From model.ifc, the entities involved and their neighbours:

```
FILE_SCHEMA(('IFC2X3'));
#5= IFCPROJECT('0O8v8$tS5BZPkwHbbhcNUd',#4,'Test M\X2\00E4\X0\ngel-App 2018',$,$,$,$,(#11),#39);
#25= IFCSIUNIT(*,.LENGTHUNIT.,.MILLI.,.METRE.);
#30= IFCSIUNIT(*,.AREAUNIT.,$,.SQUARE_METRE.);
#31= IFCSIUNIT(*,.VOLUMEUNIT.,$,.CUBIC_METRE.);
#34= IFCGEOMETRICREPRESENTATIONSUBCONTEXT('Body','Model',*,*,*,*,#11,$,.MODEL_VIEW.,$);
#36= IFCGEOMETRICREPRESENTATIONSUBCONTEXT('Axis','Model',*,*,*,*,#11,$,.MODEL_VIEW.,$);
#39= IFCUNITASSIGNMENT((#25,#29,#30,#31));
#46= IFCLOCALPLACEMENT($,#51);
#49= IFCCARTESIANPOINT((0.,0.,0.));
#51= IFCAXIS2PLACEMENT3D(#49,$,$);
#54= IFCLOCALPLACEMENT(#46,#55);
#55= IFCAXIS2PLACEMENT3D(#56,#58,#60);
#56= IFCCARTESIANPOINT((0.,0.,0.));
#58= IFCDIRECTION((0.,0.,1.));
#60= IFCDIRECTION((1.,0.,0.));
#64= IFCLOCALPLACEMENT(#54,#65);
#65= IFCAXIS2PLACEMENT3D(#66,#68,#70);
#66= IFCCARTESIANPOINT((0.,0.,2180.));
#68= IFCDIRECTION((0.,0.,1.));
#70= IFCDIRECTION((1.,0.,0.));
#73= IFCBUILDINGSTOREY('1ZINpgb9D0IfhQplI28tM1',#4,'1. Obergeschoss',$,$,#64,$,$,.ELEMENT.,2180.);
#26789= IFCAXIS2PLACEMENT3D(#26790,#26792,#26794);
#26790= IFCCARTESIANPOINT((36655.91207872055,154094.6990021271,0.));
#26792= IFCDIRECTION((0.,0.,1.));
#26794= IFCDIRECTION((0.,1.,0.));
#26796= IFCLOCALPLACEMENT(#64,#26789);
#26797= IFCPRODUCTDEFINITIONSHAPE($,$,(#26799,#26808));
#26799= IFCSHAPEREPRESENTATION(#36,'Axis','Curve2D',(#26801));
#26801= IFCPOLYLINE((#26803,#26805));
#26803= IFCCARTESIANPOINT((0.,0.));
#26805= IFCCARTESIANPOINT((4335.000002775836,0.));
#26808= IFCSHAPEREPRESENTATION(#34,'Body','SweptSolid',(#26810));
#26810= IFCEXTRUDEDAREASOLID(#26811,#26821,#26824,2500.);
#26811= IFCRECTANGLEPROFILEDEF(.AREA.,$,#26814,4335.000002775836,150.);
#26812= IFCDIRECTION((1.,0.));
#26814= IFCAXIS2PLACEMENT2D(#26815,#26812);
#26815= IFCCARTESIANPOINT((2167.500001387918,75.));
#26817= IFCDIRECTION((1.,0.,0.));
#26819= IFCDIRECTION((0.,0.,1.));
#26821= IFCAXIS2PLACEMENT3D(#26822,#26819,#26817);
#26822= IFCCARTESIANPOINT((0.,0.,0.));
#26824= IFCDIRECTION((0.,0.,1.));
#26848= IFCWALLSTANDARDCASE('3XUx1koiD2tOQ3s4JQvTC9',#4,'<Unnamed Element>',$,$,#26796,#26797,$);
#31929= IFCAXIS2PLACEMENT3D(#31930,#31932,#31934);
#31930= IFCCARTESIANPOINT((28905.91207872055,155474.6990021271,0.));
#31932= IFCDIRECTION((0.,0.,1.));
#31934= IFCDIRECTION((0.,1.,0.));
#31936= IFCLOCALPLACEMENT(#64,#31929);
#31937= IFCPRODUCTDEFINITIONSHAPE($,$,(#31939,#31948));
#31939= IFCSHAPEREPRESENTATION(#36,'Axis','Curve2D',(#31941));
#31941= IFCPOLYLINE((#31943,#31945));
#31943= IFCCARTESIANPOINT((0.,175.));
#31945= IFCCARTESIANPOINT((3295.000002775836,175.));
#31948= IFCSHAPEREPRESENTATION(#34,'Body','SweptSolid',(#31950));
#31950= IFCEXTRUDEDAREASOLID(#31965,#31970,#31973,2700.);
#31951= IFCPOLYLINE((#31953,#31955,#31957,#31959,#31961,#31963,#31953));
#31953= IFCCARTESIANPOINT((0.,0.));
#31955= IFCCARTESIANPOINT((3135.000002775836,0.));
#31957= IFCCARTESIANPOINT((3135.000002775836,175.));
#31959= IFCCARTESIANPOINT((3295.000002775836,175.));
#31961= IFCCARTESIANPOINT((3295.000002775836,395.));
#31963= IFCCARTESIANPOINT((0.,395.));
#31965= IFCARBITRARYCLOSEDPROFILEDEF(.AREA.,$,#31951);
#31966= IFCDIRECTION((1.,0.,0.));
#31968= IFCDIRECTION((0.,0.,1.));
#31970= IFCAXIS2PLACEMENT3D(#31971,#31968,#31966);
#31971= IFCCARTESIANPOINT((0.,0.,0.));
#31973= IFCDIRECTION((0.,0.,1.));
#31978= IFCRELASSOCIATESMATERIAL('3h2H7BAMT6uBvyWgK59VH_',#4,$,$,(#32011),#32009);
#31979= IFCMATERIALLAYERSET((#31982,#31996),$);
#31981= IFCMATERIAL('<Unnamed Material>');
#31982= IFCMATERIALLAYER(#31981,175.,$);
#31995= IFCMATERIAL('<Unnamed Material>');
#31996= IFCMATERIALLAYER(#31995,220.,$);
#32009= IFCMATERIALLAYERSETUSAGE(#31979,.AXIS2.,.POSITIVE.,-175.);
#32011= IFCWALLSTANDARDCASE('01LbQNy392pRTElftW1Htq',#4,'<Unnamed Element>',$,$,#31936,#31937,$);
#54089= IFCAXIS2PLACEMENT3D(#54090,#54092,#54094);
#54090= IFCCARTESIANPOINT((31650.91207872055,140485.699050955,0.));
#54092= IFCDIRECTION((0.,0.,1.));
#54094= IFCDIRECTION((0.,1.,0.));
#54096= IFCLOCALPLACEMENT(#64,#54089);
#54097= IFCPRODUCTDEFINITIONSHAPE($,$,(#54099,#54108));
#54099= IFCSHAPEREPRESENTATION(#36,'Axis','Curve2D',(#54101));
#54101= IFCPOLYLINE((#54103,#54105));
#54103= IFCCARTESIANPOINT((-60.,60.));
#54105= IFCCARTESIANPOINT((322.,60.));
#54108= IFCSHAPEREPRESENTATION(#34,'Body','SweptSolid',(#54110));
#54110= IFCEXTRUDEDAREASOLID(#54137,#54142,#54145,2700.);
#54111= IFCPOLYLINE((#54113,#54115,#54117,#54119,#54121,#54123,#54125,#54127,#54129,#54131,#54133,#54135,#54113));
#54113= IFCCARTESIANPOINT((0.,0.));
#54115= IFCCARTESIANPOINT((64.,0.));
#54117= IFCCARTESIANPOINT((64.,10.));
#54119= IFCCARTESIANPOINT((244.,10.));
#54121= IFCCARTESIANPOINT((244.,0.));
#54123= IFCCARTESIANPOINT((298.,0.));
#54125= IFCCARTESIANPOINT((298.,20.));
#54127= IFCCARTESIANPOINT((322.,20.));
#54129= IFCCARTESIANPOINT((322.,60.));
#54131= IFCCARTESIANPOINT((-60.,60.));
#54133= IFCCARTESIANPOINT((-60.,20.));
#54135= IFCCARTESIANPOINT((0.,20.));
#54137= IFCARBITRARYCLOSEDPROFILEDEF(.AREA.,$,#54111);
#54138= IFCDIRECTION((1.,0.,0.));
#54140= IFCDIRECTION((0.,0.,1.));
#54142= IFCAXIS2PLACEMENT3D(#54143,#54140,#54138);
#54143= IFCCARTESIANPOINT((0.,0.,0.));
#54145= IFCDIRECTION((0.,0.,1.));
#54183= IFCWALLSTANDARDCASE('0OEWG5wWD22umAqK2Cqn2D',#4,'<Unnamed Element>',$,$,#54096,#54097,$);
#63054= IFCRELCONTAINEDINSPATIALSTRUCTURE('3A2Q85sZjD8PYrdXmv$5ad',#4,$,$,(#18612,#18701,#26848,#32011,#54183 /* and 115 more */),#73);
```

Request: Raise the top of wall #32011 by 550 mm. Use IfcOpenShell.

```python
import ifcopenshell
import ifcopenshell.geom
import ifcopenshell.util.representation
import ifcopenshell.util.shape
import ifcopenshell.util.unit

model = ifcopenshell.open("model.ifc")
unit_scale = ifcopenshell.util.unit.calculate_unit_scale(model)
settings = ifcopenshell.geom.settings()


def volume(element):
    """Net volume in cubic metres, openings subtracted."""
    shape = ifcopenshell.geom.create_shape(settings, element)
    return ifcopenshell.util.shape.get_volume(shape.geometry)


wall = model.by_guid("01LbQNy392pRTElftW1Htq")
before = volume(wall)

body = ifcopenshell.util.representation.get_representation(wall, "Model", "Body")
solid = body.Items[0]
old_height = solid.Depth
solid.Depth += 0.55 / unit_scale
after = volume(wall)

print(f"height {old_height:g} -> {solid.Depth:g}, volume {before:.3f} -> {after:.3f} m3")

model.write("model_updated.ifc")
```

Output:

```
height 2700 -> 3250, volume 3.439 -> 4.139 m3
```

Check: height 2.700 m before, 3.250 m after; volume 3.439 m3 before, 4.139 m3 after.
